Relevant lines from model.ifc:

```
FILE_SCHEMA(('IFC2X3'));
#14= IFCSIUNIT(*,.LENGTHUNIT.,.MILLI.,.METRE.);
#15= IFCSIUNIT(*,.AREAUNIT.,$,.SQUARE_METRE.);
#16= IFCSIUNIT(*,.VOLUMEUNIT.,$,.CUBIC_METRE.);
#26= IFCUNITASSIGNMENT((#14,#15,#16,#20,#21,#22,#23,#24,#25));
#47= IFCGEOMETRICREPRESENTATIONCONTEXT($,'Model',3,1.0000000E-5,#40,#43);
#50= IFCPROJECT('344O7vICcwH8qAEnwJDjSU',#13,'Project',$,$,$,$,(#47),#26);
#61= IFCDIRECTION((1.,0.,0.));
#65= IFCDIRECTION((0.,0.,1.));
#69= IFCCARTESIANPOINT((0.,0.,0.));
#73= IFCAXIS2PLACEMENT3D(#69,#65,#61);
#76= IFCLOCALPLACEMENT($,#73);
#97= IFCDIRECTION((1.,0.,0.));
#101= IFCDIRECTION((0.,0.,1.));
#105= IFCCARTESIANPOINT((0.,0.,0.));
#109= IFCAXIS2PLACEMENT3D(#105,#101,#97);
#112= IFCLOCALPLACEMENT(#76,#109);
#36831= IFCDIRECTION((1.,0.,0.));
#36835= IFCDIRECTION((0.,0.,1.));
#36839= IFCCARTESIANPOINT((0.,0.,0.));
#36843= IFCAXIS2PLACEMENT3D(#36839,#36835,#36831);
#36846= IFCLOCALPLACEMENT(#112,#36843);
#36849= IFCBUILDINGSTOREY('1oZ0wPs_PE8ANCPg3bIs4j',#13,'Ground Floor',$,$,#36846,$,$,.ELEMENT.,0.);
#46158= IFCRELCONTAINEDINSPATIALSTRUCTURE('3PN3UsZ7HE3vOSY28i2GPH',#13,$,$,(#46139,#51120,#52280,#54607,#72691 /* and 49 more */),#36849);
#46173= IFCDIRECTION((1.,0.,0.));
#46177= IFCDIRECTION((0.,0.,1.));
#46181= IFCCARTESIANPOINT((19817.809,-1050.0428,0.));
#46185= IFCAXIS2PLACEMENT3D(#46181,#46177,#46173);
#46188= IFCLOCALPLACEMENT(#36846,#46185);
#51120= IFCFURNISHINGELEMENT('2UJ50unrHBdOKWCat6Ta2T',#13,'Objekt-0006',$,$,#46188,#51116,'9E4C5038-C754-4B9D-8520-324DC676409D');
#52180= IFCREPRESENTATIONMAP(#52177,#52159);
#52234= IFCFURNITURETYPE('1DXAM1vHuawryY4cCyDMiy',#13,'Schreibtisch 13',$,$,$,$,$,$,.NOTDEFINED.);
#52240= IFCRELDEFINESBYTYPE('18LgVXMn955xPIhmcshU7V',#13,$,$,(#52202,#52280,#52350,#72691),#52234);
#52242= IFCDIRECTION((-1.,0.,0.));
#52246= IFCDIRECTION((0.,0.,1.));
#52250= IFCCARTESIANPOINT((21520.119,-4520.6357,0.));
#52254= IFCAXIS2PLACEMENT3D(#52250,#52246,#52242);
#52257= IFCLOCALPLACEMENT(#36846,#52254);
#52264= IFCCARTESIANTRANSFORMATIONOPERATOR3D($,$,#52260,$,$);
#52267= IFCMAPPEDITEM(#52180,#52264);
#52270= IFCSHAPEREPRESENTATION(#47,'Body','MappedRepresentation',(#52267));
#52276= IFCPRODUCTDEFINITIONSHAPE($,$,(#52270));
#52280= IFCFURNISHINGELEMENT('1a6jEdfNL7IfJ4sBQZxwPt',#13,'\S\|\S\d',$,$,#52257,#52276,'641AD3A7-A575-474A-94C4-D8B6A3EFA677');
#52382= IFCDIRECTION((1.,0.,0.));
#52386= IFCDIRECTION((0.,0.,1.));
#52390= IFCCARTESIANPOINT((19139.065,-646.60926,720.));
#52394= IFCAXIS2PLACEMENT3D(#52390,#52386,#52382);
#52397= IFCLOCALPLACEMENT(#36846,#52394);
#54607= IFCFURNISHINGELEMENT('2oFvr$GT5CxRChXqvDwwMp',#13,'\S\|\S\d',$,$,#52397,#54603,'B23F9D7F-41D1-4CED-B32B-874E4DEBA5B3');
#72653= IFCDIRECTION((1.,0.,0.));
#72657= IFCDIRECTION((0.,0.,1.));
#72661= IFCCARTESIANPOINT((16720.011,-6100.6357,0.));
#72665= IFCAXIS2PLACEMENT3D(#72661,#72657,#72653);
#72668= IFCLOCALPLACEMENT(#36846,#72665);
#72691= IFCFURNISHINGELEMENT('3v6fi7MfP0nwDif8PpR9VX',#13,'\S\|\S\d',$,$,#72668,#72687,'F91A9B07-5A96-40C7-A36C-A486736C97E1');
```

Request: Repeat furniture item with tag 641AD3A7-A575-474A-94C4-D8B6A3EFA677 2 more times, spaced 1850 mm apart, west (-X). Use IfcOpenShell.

```python
import numpy as np
import ifcopenshell
import ifcopenshell.api.geometry
import ifcopenshell.api.root
import ifcopenshell.util.element
import ifcopenshell.util.placement
import ifcopenshell.util.unit

model = ifcopenshell.open("model.ifc")
unit_scale = ifcopenshell.util.unit.calculate_unit_scale(model)


def reuse_history(source, copy):
    """copy_class also copies each property set's owner history, people and application; keep the originals."""
    for rel in copy.IsDefinedBy:
        if rel.is_a("IfcRelDefinesByProperties") and (history := rel.RelatingPropertyDefinition.OwnerHistory):
            rel.RelatingPropertyDefinition.OwnerHistory = source.OwnerHistory
            ifcopenshell.util.element.remove_deep2(model, history)


source = model.by_id(52280)
base = ifcopenshell.util.placement.get_local_placement(source.ObjectPlacement)
step = np.array([-1.0, 0.0, 0.0]) * 1.85 / unit_scale

for i in range(1, 3):
    copy = ifcopenshell.api.root.copy_class(model, product=source)
    copy.Representation = ifcopenshell.util.element.copy_deep(
        model, source.Representation, exclude=["IfcGeometricRepresentationContext", "IfcRepresentationMap"]
    )
    copy.Tag = None
    reuse_history(source, copy)
    matrix = base.copy()
    matrix[:3, 3] += i * step
    print("added at", matrix[:3, 3].round(3) + 0.0)
    ifcopenshell.api.geometry.edit_object_placement(model, product=copy, matrix=matrix, is_si=False)

model.write("model_updated.ifc")
```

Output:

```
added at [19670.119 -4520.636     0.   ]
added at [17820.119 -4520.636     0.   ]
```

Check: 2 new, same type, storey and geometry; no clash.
